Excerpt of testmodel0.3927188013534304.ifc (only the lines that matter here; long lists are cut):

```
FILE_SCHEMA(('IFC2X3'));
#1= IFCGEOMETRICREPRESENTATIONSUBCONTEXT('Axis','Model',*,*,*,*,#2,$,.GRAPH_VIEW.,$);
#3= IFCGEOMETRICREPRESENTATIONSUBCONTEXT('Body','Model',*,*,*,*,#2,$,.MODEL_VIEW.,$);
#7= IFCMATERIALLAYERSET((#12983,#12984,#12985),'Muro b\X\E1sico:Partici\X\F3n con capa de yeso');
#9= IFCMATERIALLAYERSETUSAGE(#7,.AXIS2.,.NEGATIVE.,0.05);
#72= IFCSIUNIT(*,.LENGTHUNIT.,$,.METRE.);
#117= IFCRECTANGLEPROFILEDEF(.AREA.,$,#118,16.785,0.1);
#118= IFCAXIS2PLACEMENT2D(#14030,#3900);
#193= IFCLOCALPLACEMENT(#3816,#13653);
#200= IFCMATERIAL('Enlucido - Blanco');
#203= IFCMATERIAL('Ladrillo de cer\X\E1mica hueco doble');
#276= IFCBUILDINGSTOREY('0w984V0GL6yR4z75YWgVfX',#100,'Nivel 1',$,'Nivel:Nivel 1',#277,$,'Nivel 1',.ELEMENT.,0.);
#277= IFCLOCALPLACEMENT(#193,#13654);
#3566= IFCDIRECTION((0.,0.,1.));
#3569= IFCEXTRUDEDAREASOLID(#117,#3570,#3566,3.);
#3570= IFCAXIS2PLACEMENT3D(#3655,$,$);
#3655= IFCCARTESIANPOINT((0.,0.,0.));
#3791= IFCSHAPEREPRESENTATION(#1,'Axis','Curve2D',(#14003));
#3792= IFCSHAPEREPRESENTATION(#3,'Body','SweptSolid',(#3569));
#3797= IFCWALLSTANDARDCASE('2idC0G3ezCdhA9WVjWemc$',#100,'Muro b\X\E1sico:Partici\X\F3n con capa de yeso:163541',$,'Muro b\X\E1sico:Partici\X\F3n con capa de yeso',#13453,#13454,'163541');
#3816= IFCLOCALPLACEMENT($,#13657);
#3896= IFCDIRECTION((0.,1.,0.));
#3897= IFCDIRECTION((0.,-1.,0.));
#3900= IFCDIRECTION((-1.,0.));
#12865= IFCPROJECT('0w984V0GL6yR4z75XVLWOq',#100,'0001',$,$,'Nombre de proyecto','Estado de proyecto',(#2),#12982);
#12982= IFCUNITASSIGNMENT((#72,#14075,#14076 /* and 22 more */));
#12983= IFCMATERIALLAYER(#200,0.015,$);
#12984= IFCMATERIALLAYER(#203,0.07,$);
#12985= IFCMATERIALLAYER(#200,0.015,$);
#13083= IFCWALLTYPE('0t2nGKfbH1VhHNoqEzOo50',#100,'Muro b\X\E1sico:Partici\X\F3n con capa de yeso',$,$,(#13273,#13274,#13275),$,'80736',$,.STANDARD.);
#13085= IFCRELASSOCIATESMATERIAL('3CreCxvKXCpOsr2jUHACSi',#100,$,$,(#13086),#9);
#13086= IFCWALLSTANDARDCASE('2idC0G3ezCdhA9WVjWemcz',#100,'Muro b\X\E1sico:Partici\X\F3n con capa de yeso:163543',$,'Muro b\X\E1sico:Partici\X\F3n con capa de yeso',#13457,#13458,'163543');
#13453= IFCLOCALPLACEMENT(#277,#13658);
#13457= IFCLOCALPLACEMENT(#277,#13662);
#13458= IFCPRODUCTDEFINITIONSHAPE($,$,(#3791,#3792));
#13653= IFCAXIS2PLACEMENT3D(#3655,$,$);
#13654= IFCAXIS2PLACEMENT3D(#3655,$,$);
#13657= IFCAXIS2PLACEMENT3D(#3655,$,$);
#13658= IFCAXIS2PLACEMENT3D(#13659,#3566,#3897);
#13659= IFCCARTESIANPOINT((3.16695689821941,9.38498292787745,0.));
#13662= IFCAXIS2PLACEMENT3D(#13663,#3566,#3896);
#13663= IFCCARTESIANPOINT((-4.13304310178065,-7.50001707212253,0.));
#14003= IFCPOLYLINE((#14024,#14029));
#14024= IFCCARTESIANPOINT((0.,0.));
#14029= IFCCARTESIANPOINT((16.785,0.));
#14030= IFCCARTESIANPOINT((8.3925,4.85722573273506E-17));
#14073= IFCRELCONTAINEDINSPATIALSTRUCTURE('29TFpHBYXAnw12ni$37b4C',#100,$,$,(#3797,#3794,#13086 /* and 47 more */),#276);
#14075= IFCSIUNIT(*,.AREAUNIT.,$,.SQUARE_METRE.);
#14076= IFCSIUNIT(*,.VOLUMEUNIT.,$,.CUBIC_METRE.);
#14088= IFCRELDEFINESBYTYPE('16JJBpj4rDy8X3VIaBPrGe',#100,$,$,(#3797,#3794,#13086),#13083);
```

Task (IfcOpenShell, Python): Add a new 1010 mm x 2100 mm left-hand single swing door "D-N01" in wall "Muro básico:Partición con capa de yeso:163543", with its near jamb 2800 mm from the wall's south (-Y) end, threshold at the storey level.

```python
import numpy as np
import ifcopenshell
import ifcopenshell.api.feature
import ifcopenshell.api.geometry
import ifcopenshell.api.root
import ifcopenshell.api.spatial
import ifcopenshell.api.type
import ifcopenshell.geom
import ifcopenshell.util.element
import ifcopenshell.util.placement
import ifcopenshell.util.representation
import ifcopenshell.util.shape
import ifcopenshell.util.unit

model = ifcopenshell.open("testmodel0.3927188013534304.ifc")
unit_scale = ifcopenshell.util.unit.calculate_unit_scale(model)
settings = ifcopenshell.geom.settings()


def volume(element):
    """Net volume in cubic metres, openings subtracted."""
    shape = ifcopenshell.geom.create_shape(settings, element)
    return ifcopenshell.util.shape.get_volume(shape.geometry)


wall = model.by_id(13086)
storey = ifcopenshell.util.element.get_container(wall, ifc_class="IfcBuildingStorey")
context = ifcopenshell.util.representation.get_context(model, "Model", "Body", "MODEL_VIEW")
before = volume(wall)

width, height, from_end, sill = 1.01, 2.1, 2.8, 0.0  # metres

# The wall runs along its own X axis, and the end named is its -X end.
wall_shape = ifcopenshell.geom.create_shape(settings, wall)
x, y, z = ifcopenshell.util.shape.get_vertices(wall_shape.geometry).T
start = x.min() + from_end
face, thickness = float(y.min()), float(y.max() - y.min())
wall_matrix = ifcopenshell.util.placement.get_local_placement(wall.ObjectPlacement)
level = ifcopenshell.util.placement.get_local_placement(storey.ObjectPlacement)[2, 3]


def in_wall(x, y):
    """Placement at x, y metres in the wall's axes, at sill height."""
    matrix = wall_matrix.copy()
    matrix[:, 3] = wall_matrix @ np.array([x / unit_scale, y / unit_scale, 0.0, 1.0])
    matrix[2, 3] = level + sill / unit_scale
    return matrix


# Opening: a box that overshoots both wall faces by 50 mm.
opening = ifcopenshell.api.root.create_entity(model, ifc_class="IfcOpeningElement")
box = ifcopenshell.api.geometry.add_wall_representation(
    model, context=context, length=width, height=height, thickness=thickness + 0.1
)
ifcopenshell.api.geometry.assign_representation(model, product=opening, representation=box)
ifcopenshell.api.geometry.edit_object_placement(model, product=opening, matrix=in_wall(start, face - 0.05), is_si=False)
ifcopenshell.api.feature.add_feature(model, feature=opening, element=wall)

door = ifcopenshell.api.root.create_entity(model, ifc_class="IfcDoor", name="D-N01")
door.OverallWidth, door.OverallHeight = width / unit_scale, height / unit_scale
body = ifcopenshell.api.geometry.add_door_representation(
    model,
    context=context,
    overall_width=door.OverallWidth,
    overall_height=door.OverallHeight,
    operation_type="SINGLE_SWING_LEFT",
    lining_properties={"LiningDepth": thickness / unit_scale, "ThresholdDepth": thickness / unit_scale},
)
ifcopenshell.api.geometry.assign_representation(model, product=door, representation=body)
ifcopenshell.api.spatial.assign_container(model, products=[door], relating_structure=storey)
fills = ifcopenshell.api.feature.add_filling(model, opening=opening, element=door)
fills.OwnerHistory = door.OwnerHistory  # required in IFC2X3

# IFC2X3 keeps the operation on the door style.
style = ifcopenshell.api.root.create_entity(model, ifc_class="IfcDoorStyle", name="D-N01")
style.OperationType, style.ConstructionType = "SINGLE_SWING_LEFT", "NOTDEFINED"
style.ParameterTakesPrecedence = style.Sizeable = False
ifcopenshell.api.type.assign_type(model, related_objects=[door], relating_type=style)

# The lining spans the wall, so the door starts at the wall face.
ifcopenshell.api.geometry.edit_object_placement(model, product=door, matrix=in_wall(start, face), is_si=False)

after = volume(wall)

print(f"wall volume {before:.3f} -> {after:.3f} m3")

model.write("testmodel0.3927188013534304_v2.ifc")
```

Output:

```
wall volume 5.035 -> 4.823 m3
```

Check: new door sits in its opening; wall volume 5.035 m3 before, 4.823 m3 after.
